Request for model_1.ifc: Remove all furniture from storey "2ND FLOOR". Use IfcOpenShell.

First a look at what the model holds.

```python
import ifcopenshell
import ifcopenshell.util.element

model = ifcopenshell.open("model_1.ifc")
print(model.schema)
storey = next(s for s in model.by_type("IfcBuildingStorey") if s.Name == "2ND FLOOR")
furniture = [e for e in ifcopenshell.util.element.get_decomposition(storey) if e.is_a("IfcFurnishingElement")]
seen = {}
for e in furniture:
    element_type = ifcopenshell.util.element.get_type(e)
    name = element_type.Name if element_type not in (None, e) else None
    seen[name] = seen.get(name, 0) + 1
for name, count in sorted(seen.items(), key=str):
    print(count, "x", name)
```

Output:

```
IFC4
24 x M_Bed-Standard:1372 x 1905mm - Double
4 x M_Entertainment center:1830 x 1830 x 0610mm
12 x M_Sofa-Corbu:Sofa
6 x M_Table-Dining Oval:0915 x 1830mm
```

```python
import ifcopenshell
import ifcopenshell.api.root
import ifcopenshell.util.element

model = ifcopenshell.open("model_1.ifc")

storey = next(s for s in model.by_type("IfcBuildingStorey") if s.Name == "2ND FLOOR")
furniture = [e for e in ifcopenshell.util.element.get_decomposition(storey) if e.is_a("IfcFurnishingElement")]

for e in furniture:
    ifcopenshell.api.root.remove_product(model, product=e)
print(len(furniture), "removed")

model.write("model_1_updated.ifc")
```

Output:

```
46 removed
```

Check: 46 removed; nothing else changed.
